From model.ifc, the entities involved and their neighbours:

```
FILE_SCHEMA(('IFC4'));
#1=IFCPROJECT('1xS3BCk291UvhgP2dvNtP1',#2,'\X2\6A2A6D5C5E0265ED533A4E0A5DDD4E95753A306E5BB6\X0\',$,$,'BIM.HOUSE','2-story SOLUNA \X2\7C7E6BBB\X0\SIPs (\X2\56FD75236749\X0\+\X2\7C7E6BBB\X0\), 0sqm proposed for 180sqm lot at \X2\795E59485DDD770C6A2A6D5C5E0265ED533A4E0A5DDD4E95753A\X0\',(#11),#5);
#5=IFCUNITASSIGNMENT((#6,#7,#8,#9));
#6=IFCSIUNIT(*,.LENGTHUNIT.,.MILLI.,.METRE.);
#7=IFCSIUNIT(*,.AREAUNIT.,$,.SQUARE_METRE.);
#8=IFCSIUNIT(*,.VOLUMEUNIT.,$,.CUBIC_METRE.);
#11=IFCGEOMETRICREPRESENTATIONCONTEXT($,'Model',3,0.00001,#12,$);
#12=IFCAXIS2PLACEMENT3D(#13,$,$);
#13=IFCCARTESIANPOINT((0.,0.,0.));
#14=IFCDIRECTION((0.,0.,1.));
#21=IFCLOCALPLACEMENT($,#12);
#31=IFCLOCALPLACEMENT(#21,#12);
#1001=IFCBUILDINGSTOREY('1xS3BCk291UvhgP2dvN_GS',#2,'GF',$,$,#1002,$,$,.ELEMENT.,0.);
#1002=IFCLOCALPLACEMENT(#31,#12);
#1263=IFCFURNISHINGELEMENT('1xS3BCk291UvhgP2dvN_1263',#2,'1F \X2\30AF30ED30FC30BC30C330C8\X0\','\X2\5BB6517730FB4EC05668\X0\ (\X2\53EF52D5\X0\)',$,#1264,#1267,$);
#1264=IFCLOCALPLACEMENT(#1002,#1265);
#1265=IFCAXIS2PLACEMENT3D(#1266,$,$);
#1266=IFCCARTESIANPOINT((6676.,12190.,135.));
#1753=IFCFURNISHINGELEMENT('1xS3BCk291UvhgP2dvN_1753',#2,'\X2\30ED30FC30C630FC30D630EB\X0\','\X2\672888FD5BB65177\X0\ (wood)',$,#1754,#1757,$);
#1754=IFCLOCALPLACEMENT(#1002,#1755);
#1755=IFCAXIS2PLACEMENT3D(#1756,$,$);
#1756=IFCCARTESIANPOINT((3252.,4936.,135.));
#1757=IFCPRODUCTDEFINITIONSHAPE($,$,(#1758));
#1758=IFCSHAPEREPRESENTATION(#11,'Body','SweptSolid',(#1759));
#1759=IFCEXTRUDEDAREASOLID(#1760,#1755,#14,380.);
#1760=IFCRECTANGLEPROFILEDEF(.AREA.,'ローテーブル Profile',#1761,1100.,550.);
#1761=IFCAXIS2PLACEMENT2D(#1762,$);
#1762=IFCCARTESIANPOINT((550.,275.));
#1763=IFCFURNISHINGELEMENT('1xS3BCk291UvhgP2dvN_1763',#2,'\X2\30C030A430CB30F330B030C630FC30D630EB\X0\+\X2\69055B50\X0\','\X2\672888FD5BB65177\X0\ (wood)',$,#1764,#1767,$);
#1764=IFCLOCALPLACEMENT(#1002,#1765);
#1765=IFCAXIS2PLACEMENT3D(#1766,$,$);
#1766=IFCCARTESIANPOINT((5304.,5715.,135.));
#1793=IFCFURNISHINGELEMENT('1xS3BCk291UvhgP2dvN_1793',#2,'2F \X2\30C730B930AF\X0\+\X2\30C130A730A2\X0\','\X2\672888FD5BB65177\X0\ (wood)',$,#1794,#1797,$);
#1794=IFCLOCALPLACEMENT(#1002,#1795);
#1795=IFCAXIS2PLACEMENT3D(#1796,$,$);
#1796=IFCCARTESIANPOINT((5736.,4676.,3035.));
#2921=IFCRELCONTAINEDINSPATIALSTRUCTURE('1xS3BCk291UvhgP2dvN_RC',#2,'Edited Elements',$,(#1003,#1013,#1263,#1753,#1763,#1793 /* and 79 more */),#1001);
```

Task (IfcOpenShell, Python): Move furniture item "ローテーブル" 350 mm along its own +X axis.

```python
import ifcopenshell
import ifcopenshell.api.geometry
import ifcopenshell.util.placement

model = ifcopenshell.open("model.ifc")

item = model.by_guid("1xS3BCk291UvhgP2dvN_1753")
matrix = ifcopenshell.util.placement.get_local_placement(item.ObjectPlacement)
matrix[:3, 3] += matrix[:3, 0] * 350.0
ifcopenshell.api.geometry.edit_object_placement(model, product=item, matrix=matrix, is_si=False)

print(ifcopenshell.util.placement.get_local_placement(item.ObjectPlacement).round(3) + 0.0)

model.write("model_rev.ifc")
```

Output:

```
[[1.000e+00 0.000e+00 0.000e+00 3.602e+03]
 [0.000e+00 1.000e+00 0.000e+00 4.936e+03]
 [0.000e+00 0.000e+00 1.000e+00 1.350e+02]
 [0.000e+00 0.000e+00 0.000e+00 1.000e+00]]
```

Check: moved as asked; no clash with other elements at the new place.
